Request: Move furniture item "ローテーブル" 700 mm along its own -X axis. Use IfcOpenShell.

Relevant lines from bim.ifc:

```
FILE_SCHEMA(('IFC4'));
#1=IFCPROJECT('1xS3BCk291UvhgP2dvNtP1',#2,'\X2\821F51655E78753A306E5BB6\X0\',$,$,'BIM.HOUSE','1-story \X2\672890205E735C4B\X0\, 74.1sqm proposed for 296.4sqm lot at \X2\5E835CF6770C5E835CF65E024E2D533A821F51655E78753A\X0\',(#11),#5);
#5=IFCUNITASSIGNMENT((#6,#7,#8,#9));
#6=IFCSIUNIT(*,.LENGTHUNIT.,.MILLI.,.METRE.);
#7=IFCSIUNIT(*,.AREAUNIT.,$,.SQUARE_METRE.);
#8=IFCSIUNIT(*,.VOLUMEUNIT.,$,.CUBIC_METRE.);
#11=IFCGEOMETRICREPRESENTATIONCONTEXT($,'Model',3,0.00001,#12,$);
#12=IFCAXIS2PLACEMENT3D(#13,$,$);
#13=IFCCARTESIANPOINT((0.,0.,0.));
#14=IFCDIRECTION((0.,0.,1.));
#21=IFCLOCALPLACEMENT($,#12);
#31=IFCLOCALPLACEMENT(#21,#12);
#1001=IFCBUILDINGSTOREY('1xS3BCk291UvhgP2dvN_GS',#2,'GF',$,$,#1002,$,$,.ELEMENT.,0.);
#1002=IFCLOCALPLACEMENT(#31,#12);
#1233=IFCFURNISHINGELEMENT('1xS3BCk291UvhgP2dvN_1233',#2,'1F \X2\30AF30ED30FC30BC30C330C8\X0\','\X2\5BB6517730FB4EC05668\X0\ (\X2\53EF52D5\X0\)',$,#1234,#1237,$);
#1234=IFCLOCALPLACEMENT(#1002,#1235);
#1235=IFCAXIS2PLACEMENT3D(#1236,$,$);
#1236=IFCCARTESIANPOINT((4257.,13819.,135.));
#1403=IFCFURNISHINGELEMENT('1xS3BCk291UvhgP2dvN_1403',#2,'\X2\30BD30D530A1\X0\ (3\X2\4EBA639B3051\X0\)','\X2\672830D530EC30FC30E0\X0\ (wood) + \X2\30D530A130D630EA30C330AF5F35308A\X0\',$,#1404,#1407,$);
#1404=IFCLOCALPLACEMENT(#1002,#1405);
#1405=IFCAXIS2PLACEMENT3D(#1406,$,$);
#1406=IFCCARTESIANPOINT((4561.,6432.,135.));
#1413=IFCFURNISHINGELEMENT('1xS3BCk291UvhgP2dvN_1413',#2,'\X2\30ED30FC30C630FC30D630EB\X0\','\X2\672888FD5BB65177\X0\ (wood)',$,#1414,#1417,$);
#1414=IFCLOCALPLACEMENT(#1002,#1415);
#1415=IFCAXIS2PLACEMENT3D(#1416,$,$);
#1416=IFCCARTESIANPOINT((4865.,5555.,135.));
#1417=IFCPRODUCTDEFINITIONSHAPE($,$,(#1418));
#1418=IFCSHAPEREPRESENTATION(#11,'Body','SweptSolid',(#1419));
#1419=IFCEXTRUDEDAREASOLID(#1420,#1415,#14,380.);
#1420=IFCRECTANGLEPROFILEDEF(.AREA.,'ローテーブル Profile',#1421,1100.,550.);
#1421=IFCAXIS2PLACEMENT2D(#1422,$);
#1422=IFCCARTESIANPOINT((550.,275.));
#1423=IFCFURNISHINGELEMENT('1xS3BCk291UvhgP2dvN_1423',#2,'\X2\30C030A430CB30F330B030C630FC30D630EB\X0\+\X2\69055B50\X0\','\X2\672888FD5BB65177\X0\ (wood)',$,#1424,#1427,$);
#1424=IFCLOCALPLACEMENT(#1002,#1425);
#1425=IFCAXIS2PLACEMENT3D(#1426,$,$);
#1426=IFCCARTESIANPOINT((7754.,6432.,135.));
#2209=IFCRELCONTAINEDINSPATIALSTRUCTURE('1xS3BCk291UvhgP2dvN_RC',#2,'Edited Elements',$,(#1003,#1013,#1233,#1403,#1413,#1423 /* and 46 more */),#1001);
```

```python
import ifcopenshell
import ifcopenshell.api.geometry
import ifcopenshell.util.placement
import ifcopenshell.util.unit

model = ifcopenshell.open("bim.ifc")
unit_scale = ifcopenshell.util.unit.calculate_unit_scale(model)

item = model.by_guid("1xS3BCk291UvhgP2dvN_1413")
matrix = ifcopenshell.util.placement.get_local_placement(item.ObjectPlacement)
matrix[:3, 3] -= matrix[:3, 0] * 0.7 / unit_scale
ifcopenshell.api.geometry.edit_object_placement(model, product=item, matrix=matrix, is_si=False)

print(ifcopenshell.util.placement.get_local_placement(item.ObjectPlacement).round(3) + 0.0)

model.write("bim_updated.ifc")
```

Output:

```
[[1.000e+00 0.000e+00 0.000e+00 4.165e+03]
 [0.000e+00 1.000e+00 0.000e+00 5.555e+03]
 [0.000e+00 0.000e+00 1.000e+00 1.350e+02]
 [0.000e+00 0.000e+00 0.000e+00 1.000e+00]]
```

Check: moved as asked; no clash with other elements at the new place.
